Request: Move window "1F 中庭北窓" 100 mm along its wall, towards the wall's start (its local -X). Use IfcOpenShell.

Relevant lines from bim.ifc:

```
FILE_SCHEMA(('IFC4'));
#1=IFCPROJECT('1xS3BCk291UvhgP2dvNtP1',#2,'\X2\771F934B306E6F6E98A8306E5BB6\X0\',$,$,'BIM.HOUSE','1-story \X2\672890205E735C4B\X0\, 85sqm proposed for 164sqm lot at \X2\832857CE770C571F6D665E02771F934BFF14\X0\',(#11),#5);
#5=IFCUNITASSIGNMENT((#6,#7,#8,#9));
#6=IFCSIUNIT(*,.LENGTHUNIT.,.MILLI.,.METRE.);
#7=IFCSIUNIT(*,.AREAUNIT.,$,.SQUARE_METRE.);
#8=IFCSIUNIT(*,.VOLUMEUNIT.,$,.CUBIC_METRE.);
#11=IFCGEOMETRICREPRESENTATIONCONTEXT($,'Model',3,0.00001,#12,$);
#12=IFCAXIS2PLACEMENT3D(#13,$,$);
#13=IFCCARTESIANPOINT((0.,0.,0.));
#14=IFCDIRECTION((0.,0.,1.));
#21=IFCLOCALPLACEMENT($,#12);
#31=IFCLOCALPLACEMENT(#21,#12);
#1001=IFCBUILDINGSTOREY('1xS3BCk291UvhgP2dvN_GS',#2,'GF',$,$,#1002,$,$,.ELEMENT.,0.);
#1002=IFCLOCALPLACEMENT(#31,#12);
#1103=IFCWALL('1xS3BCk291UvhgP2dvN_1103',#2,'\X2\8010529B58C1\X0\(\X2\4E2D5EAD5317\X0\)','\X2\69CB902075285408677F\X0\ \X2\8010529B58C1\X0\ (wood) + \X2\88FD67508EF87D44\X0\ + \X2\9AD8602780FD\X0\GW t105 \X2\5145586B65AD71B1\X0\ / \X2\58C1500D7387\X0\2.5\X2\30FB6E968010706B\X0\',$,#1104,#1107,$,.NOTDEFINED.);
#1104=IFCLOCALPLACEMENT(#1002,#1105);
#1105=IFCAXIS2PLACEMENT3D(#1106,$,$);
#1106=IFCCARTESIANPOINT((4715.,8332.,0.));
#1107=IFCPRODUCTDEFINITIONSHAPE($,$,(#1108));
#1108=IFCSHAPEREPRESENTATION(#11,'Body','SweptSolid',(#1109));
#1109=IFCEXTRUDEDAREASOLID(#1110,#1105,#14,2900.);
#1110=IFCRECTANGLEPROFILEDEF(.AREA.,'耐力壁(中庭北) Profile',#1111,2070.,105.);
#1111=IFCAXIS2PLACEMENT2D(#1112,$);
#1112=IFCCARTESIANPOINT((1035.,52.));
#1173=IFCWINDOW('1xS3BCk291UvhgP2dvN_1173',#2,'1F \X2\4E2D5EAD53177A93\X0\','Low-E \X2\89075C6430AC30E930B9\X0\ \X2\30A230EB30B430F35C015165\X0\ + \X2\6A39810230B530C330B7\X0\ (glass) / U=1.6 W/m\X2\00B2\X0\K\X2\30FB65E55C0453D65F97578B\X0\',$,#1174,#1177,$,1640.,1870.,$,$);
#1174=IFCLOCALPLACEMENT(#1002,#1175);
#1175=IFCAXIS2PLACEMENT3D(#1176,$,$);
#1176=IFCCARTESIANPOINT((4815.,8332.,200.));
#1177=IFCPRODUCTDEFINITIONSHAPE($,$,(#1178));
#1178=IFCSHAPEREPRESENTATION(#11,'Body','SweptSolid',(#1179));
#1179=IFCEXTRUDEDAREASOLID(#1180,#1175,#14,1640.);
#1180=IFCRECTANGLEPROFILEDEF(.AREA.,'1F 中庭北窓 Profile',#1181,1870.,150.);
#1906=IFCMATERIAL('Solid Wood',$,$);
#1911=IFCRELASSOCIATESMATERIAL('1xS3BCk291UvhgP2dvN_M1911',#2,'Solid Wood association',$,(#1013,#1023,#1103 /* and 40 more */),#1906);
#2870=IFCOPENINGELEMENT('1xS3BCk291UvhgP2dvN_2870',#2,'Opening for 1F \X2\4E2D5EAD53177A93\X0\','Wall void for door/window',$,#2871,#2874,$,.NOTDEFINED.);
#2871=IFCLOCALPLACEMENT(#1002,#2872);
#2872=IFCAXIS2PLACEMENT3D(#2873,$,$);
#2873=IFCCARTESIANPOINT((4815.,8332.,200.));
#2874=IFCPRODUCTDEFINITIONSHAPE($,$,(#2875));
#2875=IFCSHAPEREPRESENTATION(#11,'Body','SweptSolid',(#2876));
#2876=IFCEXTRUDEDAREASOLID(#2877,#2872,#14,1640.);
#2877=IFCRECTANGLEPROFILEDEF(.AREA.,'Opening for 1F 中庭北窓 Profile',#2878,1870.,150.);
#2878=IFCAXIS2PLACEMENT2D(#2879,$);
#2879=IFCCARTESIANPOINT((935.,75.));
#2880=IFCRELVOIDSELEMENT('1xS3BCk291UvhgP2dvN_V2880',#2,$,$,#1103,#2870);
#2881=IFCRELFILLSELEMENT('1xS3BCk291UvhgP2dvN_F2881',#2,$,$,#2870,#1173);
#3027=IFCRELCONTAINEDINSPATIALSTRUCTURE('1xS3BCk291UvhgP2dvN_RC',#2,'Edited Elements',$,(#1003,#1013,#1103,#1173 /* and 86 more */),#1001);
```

```python
import ifcopenshell
import ifcopenshell.api.geometry
import ifcopenshell.util.placement
import ifcopenshell.util.unit

model = ifcopenshell.open("bim.ifc")
unit_scale = ifcopenshell.util.unit.calculate_unit_scale(model)

window = model.by_guid("1xS3BCk291UvhgP2dvN_1173")
opening = window.FillsVoids[0].RelatingOpeningElement
wall = opening.VoidsElements[0].RelatingBuildingElement

wall_matrix = ifcopenshell.util.placement.get_local_placement(wall.ObjectPlacement)
shift = wall_matrix[:3, 0] * -0.1 / unit_scale
before = ifcopenshell.util.placement.get_local_placement(window.ObjectPlacement)[:3, 3].copy()

# The window is not placed relative to its opening, so move both.
for product in (opening, window):
    matrix = ifcopenshell.util.placement.get_local_placement(product.ObjectPlacement)
    matrix[:3, 3] += shift
    ifcopenshell.api.geometry.edit_object_placement(model, product=product, matrix=matrix, is_si=False)

after = ifcopenshell.util.placement.get_local_placement(window.ObjectPlacement)[:3, 3]
print("window moved by", (after - before).round(3) + 0.0)

model.write("bim_edited.ifc")
```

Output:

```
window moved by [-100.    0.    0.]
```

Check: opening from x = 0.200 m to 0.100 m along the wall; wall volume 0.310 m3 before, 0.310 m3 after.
